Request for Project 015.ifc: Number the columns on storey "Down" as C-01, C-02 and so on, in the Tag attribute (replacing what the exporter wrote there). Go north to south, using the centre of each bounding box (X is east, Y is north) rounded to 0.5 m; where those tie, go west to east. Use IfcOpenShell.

First a look at what the model holds.

```python
import ifcopenshell
import ifcopenshell.util.element
import ifcopenshell.util.placement

model = ifcopenshell.open("Project 015.ifc")
print(model.schema)
storey = next(s for s in model.by_type("IfcBuildingStorey") if s.Name == "Down")
columns = [e for e in ifcopenshell.util.element.get_decomposition(storey) if e.is_a("IfcColumn")]
for e in sorted(columns, key=lambda e: e.id()):
    origin = ifcopenshell.util.placement.get_local_placement(e.ObjectPlacement)[:3, 3]
    print(e.id(), e.Tag, e.Name, origin.round(2) + 0.0, sep=" | ")
```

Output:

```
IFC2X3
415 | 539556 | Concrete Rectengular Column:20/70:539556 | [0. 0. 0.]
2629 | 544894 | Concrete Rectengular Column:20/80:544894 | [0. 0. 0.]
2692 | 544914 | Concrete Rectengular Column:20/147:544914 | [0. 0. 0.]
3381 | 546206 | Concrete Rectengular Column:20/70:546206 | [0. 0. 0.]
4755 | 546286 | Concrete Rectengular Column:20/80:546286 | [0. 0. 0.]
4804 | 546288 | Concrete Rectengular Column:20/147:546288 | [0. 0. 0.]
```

```python
import ifcopenshell
import ifcopenshell.geom
import ifcopenshell.util.element
import ifcopenshell.util.shape

model = ifcopenshell.open("Project 015.ifc")
settings = ifcopenshell.geom.settings()
settings.set("use-world-coords", True)


def centre(element):
    shape = ifcopenshell.geom.create_shape(settings, element)
    return ifcopenshell.util.shape.get_bbox_centroid(shape.geometry)


storey = next(s for s in model.by_type("IfcBuildingStorey") if s.Name == "Down")
columns = [e for e in ifcopenshell.util.element.get_decomposition(storey) if e.is_a("IfcColumn")]

# Insertion points can sit at a corner or the storey origin, so sort by the geometry (in metres).
centres = {e: centre(e) for e in columns}
columns.sort(key=lambda e: (-round(centres[e][1] / 0.5), centres[e][0]))

for i, e in enumerate(columns, start=1):
    number = f"C-{i:02d}"
    e.Tag = number
    print(e.id(), number)

model.write("Project 015_rev.ifc")
```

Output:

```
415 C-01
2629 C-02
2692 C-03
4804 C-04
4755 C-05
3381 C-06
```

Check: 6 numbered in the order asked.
